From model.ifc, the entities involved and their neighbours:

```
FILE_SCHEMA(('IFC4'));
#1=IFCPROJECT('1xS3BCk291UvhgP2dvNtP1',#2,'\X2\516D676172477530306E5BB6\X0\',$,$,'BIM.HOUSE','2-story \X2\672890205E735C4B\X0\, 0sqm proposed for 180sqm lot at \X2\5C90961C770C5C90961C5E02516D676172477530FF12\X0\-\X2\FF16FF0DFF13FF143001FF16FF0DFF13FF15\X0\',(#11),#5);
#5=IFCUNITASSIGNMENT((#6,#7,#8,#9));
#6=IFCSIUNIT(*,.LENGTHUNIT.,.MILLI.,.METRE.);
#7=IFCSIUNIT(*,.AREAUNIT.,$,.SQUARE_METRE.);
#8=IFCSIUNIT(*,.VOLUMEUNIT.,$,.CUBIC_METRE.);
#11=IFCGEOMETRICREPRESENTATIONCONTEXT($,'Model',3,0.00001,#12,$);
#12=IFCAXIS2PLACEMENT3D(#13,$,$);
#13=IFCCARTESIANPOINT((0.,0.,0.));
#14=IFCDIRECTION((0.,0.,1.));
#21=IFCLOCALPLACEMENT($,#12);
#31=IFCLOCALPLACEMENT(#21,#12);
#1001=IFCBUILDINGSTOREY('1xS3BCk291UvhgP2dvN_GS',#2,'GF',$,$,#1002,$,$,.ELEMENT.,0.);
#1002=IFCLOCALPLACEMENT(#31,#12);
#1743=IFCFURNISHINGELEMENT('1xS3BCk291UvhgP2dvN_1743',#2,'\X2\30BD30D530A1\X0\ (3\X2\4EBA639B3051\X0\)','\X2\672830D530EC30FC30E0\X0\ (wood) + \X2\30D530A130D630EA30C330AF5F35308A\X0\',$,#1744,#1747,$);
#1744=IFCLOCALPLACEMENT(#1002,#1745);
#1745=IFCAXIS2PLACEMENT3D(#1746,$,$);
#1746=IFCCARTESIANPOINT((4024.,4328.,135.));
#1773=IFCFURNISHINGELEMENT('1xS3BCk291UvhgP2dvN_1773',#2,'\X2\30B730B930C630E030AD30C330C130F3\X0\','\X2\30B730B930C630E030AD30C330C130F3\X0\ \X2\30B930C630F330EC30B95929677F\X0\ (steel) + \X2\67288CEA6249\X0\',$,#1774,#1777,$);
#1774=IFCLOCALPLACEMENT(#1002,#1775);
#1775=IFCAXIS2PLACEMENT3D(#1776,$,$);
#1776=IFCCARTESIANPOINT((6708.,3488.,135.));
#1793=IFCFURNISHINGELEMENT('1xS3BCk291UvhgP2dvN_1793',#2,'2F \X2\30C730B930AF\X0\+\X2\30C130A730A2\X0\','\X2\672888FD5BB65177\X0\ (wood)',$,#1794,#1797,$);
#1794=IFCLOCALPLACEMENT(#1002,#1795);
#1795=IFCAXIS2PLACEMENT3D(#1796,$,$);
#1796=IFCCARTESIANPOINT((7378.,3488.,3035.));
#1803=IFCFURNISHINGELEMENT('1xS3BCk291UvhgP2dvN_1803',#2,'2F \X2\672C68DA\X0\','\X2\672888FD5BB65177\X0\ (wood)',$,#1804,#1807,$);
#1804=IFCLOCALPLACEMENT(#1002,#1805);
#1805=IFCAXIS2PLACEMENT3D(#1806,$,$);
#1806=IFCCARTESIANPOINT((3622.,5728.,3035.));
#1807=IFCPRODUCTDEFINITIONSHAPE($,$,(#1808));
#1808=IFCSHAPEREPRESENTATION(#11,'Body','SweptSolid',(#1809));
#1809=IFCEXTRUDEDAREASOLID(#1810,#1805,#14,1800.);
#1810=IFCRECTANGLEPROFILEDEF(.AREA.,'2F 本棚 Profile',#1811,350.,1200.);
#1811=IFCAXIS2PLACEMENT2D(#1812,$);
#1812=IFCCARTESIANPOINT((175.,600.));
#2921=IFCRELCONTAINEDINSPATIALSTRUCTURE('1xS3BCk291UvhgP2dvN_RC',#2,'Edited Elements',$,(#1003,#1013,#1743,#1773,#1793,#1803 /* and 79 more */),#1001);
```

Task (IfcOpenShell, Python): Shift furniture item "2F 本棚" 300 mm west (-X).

```python
import ifcopenshell
import ifcopenshell.api.geometry
import ifcopenshell.util.placement
import ifcopenshell.util.unit

model = ifcopenshell.open("model.ifc")
unit_scale = ifcopenshell.util.unit.calculate_unit_scale(model)

item = model.by_id(1803)
matrix = ifcopenshell.util.placement.get_local_placement(item.ObjectPlacement)
matrix[0, 3] -= 0.3 / unit_scale
ifcopenshell.api.geometry.edit_object_placement(model, product=item, matrix=matrix, is_si=False)

print(ifcopenshell.util.placement.get_local_placement(item.ObjectPlacement).round(3) + 0.0)

model.write("model_rev.ifc")
```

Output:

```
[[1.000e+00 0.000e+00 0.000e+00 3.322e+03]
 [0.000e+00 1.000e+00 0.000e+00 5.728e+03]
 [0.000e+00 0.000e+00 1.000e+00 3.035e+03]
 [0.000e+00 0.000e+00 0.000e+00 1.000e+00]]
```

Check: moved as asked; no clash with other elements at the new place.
